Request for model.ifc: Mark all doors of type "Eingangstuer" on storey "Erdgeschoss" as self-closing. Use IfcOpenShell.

First a look at what the model holds.

```python
import ifcopenshell
import ifcopenshell.util.element

model = ifcopenshell.open("model.ifc")
print(model.schema)
storey = next(s for s in model.by_type("IfcBuildingStorey") if s.Name == "Erdgeschoss")
doors = [e for e in ifcopenshell.util.element.get_decomposition(storey) if e.is_a("IfcDoor")]
seen = {}
for e in doors:
    element_type = ifcopenshell.util.element.get_type(e)
    key = (element_type.Name if element_type != e and element_type else None, ifcopenshell.util.element.get_pset(e, "Pset_DoorCommon", "SelfClosing"))
    seen[key] = seen.get(key, 0) + 1
for (name, value), count in sorted(seen.items(), key=str):
    print(count, "x", name, "|", value)
```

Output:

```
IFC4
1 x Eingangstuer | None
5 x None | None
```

```python
import ifcopenshell
import ifcopenshell.api.pset
import ifcopenshell.util.element

model = ifcopenshell.open("model.ifc")

storey = next(s for s in model.by_type("IfcBuildingStorey") if s.Name == "Erdgeschoss")
doors = [e for e in ifcopenshell.util.element.get_decomposition(storey) if e.is_a("IfcDoor")]

count = 0
for e in doors:
    element_type = ifcopenshell.util.element.get_type(e)
    if element_type in (None, e) or element_type.Name != "Eingangstuer":
        continue
    # add_pset returns the element's existing set when there is one.
    pset = ifcopenshell.api.pset.add_pset(model, product=e, name="Pset_DoorCommon")
    ifcopenshell.api.pset.edit_pset(model, pset=pset, properties={"SelfClosing": True})
    count += 1

print(count, "doors updated")

model.write("model_updated.ifc")
```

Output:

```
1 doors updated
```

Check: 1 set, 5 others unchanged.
